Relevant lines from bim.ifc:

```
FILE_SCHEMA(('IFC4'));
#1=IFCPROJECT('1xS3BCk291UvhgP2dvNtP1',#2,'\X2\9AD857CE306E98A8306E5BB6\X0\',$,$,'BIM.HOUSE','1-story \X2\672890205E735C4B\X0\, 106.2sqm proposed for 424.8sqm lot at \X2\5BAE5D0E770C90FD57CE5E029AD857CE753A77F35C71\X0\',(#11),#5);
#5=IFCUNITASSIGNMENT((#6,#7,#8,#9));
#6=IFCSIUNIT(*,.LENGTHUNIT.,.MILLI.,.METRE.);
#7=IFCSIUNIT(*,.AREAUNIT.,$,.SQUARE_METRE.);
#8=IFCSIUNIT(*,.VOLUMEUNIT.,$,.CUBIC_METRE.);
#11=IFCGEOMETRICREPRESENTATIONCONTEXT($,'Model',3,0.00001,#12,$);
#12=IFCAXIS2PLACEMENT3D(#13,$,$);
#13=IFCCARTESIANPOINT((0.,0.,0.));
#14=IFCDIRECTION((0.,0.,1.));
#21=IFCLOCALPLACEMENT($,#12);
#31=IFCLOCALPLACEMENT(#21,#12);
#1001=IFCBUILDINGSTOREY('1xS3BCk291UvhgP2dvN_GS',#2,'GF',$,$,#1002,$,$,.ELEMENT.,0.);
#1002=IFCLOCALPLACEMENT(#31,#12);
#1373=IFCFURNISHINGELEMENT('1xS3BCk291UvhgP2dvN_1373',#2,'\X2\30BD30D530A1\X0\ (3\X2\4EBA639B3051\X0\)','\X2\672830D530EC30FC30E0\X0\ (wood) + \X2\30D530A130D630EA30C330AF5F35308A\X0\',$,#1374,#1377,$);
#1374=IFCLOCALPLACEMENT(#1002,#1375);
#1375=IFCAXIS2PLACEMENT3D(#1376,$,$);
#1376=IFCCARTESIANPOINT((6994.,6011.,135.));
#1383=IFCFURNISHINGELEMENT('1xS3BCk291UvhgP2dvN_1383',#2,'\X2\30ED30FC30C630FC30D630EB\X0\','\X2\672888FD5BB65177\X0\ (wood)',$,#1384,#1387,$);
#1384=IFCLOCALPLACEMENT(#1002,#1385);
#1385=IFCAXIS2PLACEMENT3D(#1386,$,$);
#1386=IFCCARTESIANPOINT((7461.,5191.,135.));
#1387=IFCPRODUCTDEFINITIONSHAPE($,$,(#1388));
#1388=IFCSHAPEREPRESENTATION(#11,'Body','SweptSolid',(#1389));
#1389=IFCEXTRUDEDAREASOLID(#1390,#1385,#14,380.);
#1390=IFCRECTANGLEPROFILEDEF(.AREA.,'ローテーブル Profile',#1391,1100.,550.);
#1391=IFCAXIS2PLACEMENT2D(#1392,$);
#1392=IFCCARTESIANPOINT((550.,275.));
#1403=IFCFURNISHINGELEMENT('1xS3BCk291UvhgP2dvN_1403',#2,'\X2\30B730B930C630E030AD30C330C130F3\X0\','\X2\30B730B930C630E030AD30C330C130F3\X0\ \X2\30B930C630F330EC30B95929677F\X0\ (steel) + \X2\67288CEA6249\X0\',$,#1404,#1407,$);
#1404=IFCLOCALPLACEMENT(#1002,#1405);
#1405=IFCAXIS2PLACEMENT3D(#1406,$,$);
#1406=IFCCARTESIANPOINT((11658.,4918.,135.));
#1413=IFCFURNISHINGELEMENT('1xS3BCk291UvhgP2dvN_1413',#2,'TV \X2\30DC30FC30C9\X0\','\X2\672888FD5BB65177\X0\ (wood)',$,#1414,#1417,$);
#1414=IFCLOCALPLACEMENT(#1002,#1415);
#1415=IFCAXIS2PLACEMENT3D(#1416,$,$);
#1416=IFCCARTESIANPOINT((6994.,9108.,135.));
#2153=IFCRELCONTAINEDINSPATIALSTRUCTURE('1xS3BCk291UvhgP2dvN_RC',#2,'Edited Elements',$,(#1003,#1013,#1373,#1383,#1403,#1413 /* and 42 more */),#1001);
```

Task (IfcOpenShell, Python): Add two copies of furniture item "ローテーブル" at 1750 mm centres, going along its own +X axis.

```python
import ifcopenshell
import ifcopenshell.api.geometry
import ifcopenshell.api.root
import ifcopenshell.util.element
import ifcopenshell.util.placement

model = ifcopenshell.open("bim.ifc")


def reuse_history(source, copy):
    """copy_class also copies each property set's owner history, people and application; keep the originals."""
    for rel in copy.IsDefinedBy:
        if rel.is_a("IfcRelDefinesByProperties") and (history := rel.RelatingPropertyDefinition.OwnerHistory):
            rel.RelatingPropertyDefinition.OwnerHistory = source.OwnerHistory
            ifcopenshell.util.element.remove_deep2(model, history)


source = model.by_id(1383)
base = ifcopenshell.util.placement.get_local_placement(source.ObjectPlacement)
step = base[:3, 0] * 1750.0

for i in range(1, 3):
    copy = ifcopenshell.api.root.copy_class(model, product=source)
    copy.Representation = ifcopenshell.util.element.copy_deep(
        model, source.Representation, exclude=["IfcGeometricRepresentationContext", "IfcRepresentationMap"]
    )
    reuse_history(source, copy)
    matrix = base.copy()
    matrix[:3, 3] += i * step
    print("added at", matrix[:3, 3].round(3) + 0.0)
    ifcopenshell.api.geometry.edit_object_placement(model, product=copy, matrix=matrix, is_si=False)

model.write("bim-out.ifc")
```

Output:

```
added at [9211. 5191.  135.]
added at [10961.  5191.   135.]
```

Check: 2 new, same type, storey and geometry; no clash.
